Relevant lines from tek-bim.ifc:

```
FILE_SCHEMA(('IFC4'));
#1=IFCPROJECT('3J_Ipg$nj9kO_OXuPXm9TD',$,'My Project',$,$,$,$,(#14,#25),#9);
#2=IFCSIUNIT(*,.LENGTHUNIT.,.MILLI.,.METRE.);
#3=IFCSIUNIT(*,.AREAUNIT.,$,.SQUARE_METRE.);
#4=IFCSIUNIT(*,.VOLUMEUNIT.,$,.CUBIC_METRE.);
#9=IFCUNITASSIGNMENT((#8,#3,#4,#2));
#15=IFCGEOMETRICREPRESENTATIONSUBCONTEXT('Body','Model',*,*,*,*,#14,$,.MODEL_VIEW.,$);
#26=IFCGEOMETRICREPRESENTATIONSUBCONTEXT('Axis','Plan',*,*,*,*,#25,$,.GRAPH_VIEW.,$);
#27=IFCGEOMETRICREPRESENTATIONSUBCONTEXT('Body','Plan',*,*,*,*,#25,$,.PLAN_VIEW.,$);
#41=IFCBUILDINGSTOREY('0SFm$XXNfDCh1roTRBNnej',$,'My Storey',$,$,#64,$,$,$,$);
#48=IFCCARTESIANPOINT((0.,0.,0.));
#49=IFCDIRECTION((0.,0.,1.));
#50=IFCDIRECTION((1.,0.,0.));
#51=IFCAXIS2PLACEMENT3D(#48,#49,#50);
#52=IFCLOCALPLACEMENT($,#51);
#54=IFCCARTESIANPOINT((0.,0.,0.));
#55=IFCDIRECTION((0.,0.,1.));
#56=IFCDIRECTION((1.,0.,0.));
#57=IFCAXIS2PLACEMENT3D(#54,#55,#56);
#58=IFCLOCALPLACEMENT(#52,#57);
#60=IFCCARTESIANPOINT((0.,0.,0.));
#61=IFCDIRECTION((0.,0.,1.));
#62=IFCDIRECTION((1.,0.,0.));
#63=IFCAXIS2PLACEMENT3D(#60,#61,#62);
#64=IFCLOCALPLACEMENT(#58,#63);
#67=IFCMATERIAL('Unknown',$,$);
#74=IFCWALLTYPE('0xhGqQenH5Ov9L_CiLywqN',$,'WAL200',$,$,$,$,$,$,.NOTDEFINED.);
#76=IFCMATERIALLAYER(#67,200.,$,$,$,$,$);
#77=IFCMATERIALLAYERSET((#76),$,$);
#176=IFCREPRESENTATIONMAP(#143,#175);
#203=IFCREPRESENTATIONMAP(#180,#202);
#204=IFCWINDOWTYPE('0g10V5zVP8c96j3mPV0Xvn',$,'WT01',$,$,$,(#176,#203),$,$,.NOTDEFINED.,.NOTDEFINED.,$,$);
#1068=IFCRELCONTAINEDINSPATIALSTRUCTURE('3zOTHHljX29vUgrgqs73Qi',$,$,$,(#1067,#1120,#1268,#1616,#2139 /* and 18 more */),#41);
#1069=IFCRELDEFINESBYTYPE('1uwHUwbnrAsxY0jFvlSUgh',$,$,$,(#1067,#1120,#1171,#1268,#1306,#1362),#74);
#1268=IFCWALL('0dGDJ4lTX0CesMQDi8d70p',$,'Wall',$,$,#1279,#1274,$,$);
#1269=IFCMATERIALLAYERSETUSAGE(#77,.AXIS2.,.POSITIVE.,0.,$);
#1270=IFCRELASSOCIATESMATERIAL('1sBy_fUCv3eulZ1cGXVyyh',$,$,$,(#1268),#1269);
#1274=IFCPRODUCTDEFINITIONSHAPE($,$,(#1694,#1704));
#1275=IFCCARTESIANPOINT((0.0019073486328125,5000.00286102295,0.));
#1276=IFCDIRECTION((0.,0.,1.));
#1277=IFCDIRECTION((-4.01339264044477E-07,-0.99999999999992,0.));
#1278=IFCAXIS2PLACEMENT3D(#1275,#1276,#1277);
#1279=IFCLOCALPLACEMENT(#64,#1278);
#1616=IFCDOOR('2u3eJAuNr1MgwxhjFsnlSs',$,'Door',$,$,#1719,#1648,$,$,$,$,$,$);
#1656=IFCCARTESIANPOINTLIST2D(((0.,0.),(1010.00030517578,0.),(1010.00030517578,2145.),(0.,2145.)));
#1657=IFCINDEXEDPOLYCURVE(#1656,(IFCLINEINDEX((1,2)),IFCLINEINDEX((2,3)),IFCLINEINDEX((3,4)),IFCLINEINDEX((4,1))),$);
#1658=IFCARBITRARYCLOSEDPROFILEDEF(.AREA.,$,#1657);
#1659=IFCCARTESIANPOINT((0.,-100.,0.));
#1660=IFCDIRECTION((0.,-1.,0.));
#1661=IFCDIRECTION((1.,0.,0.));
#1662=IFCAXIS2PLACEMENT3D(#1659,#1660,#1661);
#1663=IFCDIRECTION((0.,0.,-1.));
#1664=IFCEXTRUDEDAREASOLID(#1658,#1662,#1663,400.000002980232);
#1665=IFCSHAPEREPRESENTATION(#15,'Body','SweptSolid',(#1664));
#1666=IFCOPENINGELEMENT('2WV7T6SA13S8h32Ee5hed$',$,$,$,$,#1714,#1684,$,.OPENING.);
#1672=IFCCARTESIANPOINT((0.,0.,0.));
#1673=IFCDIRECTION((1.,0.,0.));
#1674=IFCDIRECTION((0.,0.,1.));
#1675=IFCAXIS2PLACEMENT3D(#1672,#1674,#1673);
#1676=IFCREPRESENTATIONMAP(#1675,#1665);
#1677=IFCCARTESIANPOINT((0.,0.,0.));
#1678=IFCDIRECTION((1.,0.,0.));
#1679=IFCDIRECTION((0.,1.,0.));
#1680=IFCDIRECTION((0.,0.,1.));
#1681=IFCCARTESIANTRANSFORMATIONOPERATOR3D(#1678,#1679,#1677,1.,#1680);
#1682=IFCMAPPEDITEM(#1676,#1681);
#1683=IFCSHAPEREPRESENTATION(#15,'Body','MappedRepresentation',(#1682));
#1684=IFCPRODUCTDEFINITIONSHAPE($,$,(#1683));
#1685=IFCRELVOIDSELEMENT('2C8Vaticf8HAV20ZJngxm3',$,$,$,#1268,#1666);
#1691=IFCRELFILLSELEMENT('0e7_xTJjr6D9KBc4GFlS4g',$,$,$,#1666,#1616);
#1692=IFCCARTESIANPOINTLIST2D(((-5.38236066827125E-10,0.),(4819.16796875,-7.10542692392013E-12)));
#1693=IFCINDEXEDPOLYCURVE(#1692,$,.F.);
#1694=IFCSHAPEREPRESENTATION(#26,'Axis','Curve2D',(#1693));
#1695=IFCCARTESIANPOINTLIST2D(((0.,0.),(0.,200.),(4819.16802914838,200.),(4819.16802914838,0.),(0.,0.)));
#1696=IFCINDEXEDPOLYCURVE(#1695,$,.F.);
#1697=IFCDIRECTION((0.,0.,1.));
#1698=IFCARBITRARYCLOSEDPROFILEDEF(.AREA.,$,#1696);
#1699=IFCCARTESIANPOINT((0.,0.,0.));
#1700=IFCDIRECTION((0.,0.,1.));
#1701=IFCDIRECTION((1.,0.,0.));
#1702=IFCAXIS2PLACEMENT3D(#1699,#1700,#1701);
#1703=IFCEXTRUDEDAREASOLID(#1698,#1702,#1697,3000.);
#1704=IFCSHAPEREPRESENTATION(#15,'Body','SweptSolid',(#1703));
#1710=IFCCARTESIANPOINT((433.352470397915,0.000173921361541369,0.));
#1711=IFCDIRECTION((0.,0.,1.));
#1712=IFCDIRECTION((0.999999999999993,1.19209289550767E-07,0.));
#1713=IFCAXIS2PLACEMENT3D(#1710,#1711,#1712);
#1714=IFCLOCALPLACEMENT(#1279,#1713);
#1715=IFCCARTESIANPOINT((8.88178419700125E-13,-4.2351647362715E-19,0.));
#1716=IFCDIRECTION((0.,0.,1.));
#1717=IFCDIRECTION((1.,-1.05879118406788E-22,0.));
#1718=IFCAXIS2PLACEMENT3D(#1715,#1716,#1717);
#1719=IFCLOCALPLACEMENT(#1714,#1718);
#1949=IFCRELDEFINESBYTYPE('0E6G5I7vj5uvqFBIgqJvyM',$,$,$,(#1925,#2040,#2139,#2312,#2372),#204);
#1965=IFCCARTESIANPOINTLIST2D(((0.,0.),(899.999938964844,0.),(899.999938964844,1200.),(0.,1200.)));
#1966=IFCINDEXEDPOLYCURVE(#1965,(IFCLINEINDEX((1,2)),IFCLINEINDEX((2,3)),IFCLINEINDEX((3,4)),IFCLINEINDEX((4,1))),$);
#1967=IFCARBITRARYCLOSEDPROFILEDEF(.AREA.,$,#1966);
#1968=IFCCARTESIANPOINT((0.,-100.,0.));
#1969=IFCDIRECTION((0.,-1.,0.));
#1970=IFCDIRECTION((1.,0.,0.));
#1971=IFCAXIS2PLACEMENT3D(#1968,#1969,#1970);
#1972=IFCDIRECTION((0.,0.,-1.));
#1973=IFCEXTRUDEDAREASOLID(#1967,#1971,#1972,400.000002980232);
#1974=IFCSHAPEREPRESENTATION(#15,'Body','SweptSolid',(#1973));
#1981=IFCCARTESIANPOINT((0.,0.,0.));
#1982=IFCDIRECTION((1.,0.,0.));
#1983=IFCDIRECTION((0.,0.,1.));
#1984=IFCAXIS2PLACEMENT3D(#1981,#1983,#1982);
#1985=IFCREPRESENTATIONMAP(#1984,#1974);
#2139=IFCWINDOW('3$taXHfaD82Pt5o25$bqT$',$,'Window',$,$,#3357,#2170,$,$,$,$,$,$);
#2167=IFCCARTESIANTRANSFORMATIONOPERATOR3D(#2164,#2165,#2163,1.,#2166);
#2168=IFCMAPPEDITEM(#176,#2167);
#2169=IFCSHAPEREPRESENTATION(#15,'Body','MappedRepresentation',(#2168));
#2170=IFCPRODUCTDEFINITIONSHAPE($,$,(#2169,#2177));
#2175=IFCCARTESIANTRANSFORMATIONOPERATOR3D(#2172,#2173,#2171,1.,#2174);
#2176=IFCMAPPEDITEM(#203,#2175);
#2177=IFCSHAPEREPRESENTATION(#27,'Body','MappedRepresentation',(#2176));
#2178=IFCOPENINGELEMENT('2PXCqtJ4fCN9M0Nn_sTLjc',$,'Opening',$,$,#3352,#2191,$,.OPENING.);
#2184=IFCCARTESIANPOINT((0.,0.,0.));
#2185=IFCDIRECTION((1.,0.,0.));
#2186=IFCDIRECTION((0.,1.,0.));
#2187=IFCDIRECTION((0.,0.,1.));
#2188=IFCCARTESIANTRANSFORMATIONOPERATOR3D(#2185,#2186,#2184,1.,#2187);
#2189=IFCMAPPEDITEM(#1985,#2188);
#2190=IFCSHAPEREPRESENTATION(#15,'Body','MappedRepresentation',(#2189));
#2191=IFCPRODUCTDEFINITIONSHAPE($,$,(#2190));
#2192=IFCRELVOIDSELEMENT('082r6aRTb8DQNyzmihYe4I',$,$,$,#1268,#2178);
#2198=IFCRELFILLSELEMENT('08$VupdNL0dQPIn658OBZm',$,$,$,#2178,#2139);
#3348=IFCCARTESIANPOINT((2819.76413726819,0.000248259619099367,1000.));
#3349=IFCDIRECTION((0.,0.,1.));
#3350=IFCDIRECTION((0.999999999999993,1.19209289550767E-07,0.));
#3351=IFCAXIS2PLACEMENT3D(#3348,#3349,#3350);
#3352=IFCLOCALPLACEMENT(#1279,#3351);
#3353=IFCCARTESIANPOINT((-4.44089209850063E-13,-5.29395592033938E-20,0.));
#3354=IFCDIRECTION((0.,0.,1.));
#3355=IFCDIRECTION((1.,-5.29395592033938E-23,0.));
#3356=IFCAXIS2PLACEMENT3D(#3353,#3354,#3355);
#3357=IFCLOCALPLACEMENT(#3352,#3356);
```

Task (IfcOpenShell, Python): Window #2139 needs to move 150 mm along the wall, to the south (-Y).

```python
import ifcopenshell
import ifcopenshell.api.geometry
import ifcopenshell.util.placement
import ifcopenshell.util.unit

model = ifcopenshell.open("tek-bim.ifc")
unit_scale = ifcopenshell.util.unit.calculate_unit_scale(model)

window = model.by_guid("3$taXHfaD82Pt5o25$bqT$")
opening = window.FillsVoids[0].RelatingOpeningElement
wall = opening.VoidsElements[0].RelatingBuildingElement

wall_matrix = ifcopenshell.util.placement.get_local_placement(wall.ObjectPlacement)
shift = wall_matrix[:3, 0] * 0.15 / unit_scale
before = ifcopenshell.util.placement.get_local_placement(window.ObjectPlacement)[:3, 3].copy()

# The window is placed relative to its opening, so it follows when the opening moves.
matrix = ifcopenshell.util.placement.get_local_placement(opening.ObjectPlacement)
matrix[:3, 3] += shift
ifcopenshell.api.geometry.edit_object_placement(
    model, product=opening, matrix=matrix, is_si=False, should_transform_children=True
)

after = ifcopenshell.util.placement.get_local_placement(window.ObjectPlacement)[:3, 3]
print("window moved by", (after - before).round(3) + 0.0)

model.write("tek-bim_updated.ifc")
```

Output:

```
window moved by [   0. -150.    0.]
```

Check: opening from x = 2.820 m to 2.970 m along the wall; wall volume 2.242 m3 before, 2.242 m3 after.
